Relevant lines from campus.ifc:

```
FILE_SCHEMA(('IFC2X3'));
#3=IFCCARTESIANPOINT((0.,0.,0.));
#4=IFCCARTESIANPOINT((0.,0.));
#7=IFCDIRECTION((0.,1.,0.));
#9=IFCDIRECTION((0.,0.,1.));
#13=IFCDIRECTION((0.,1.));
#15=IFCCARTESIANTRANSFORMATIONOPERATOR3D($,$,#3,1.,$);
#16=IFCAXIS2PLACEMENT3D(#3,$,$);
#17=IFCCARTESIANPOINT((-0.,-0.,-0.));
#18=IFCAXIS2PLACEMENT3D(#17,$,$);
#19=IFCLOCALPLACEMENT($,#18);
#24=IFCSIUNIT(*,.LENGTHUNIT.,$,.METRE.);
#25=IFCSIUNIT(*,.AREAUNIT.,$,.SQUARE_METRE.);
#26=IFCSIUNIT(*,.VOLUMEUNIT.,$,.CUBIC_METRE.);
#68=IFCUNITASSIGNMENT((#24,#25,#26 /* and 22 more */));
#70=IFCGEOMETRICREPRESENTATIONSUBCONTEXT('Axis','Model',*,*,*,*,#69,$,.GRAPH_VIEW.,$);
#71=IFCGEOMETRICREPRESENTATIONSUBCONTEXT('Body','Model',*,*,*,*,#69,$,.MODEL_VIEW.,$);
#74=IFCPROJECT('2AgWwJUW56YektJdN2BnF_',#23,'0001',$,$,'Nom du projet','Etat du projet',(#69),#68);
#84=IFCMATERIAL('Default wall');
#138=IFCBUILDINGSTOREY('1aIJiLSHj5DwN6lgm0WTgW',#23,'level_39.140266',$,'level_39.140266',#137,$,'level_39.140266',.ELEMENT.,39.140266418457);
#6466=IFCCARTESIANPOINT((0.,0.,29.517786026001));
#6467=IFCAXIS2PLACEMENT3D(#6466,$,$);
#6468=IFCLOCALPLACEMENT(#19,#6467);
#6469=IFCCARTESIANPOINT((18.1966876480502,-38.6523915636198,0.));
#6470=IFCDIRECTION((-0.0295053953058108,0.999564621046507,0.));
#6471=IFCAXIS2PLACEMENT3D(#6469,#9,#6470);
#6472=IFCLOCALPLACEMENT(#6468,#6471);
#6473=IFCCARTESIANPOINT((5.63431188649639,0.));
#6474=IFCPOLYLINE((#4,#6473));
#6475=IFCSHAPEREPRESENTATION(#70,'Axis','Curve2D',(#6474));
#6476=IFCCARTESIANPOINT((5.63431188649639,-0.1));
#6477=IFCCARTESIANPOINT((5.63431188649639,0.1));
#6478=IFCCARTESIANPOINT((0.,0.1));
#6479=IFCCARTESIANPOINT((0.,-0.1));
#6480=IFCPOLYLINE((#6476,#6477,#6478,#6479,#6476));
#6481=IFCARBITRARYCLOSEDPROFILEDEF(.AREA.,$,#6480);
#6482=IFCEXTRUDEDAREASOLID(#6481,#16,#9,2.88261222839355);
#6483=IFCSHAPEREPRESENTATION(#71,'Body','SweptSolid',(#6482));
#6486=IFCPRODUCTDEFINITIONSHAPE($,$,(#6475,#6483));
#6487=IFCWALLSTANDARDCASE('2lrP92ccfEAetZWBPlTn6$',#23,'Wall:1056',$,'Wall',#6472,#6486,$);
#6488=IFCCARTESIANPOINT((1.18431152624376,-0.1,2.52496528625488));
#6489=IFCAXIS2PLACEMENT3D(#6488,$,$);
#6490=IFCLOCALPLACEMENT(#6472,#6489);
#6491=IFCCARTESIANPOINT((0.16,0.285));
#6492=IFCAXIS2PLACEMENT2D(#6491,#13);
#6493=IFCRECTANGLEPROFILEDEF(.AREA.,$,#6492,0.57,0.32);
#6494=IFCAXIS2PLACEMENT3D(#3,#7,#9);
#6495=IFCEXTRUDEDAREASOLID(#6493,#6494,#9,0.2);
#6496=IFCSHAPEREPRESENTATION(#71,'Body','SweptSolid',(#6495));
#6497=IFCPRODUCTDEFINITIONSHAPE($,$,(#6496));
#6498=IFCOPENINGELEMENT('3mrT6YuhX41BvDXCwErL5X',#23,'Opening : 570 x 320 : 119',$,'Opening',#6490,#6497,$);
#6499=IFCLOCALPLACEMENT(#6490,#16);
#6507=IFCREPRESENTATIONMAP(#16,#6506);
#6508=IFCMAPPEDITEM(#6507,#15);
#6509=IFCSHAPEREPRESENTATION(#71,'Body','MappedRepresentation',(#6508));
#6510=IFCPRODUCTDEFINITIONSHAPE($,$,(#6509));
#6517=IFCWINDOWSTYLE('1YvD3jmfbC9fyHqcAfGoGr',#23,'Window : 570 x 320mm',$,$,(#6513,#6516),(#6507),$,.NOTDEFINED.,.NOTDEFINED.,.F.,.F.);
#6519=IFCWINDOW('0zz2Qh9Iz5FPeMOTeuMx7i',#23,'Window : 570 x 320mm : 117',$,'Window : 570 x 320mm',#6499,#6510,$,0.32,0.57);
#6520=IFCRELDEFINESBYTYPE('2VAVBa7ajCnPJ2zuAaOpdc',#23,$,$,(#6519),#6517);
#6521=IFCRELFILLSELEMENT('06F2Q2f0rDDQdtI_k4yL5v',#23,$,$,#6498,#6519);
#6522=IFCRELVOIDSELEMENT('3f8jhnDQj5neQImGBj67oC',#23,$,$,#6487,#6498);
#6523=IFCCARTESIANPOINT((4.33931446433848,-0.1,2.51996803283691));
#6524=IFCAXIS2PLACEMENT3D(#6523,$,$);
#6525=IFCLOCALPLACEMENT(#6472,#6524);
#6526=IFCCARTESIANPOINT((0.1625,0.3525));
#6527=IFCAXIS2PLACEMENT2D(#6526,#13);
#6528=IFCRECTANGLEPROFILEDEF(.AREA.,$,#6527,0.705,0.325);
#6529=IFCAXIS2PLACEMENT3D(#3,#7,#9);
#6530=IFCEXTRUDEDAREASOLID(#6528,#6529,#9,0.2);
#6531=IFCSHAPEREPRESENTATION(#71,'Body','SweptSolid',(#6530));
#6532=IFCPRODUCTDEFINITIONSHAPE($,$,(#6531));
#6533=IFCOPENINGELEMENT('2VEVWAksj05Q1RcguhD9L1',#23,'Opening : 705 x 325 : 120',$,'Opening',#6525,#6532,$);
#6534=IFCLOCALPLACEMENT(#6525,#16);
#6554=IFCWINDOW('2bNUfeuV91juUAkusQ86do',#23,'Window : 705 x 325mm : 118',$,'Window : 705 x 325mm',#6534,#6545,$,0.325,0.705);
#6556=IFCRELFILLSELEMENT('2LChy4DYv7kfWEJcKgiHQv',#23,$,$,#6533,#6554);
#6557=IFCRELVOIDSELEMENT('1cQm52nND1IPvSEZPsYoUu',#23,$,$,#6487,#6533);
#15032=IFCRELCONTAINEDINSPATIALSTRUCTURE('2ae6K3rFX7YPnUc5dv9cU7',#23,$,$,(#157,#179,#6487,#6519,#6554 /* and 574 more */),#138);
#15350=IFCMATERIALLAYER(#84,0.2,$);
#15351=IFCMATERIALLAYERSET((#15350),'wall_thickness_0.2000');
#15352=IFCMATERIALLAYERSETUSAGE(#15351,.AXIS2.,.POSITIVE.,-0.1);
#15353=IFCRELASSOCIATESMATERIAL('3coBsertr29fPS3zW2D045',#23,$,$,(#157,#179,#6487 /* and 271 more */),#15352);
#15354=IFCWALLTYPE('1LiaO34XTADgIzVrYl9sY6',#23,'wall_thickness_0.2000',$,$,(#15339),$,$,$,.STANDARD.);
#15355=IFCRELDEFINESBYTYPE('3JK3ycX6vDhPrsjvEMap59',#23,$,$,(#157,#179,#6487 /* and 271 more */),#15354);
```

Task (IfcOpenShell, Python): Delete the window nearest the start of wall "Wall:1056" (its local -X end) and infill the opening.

```python
import ifcopenshell
import ifcopenshell.api.feature
import ifcopenshell.api.root
import ifcopenshell.geom
import ifcopenshell.util.shape

model = ifcopenshell.open("campus.ifc")
settings = ifcopenshell.geom.settings()


def volume(element):
    """Net volume in cubic metres, openings subtracted."""
    shape = ifcopenshell.geom.create_shape(settings, element)
    return ifcopenshell.util.shape.get_volume(shape.geometry)


window = model.by_guid("0zz2Qh9Iz5FPeMOTeuMx7i")
opening = window.FillsVoids[0].RelatingOpeningElement
wall = opening.VoidsElements[0].RelatingBuildingElement
before = volume(wall)

ifcopenshell.api.root.remove_product(model, product=window)
ifcopenshell.api.feature.remove_feature(model, feature=opening)

after = volume(wall)

print(f"wall volume {before:.3f} -> {after:.3f} m3")

model.write("campus_rev.ifc")
```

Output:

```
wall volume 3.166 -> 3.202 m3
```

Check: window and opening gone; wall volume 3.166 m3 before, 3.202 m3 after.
